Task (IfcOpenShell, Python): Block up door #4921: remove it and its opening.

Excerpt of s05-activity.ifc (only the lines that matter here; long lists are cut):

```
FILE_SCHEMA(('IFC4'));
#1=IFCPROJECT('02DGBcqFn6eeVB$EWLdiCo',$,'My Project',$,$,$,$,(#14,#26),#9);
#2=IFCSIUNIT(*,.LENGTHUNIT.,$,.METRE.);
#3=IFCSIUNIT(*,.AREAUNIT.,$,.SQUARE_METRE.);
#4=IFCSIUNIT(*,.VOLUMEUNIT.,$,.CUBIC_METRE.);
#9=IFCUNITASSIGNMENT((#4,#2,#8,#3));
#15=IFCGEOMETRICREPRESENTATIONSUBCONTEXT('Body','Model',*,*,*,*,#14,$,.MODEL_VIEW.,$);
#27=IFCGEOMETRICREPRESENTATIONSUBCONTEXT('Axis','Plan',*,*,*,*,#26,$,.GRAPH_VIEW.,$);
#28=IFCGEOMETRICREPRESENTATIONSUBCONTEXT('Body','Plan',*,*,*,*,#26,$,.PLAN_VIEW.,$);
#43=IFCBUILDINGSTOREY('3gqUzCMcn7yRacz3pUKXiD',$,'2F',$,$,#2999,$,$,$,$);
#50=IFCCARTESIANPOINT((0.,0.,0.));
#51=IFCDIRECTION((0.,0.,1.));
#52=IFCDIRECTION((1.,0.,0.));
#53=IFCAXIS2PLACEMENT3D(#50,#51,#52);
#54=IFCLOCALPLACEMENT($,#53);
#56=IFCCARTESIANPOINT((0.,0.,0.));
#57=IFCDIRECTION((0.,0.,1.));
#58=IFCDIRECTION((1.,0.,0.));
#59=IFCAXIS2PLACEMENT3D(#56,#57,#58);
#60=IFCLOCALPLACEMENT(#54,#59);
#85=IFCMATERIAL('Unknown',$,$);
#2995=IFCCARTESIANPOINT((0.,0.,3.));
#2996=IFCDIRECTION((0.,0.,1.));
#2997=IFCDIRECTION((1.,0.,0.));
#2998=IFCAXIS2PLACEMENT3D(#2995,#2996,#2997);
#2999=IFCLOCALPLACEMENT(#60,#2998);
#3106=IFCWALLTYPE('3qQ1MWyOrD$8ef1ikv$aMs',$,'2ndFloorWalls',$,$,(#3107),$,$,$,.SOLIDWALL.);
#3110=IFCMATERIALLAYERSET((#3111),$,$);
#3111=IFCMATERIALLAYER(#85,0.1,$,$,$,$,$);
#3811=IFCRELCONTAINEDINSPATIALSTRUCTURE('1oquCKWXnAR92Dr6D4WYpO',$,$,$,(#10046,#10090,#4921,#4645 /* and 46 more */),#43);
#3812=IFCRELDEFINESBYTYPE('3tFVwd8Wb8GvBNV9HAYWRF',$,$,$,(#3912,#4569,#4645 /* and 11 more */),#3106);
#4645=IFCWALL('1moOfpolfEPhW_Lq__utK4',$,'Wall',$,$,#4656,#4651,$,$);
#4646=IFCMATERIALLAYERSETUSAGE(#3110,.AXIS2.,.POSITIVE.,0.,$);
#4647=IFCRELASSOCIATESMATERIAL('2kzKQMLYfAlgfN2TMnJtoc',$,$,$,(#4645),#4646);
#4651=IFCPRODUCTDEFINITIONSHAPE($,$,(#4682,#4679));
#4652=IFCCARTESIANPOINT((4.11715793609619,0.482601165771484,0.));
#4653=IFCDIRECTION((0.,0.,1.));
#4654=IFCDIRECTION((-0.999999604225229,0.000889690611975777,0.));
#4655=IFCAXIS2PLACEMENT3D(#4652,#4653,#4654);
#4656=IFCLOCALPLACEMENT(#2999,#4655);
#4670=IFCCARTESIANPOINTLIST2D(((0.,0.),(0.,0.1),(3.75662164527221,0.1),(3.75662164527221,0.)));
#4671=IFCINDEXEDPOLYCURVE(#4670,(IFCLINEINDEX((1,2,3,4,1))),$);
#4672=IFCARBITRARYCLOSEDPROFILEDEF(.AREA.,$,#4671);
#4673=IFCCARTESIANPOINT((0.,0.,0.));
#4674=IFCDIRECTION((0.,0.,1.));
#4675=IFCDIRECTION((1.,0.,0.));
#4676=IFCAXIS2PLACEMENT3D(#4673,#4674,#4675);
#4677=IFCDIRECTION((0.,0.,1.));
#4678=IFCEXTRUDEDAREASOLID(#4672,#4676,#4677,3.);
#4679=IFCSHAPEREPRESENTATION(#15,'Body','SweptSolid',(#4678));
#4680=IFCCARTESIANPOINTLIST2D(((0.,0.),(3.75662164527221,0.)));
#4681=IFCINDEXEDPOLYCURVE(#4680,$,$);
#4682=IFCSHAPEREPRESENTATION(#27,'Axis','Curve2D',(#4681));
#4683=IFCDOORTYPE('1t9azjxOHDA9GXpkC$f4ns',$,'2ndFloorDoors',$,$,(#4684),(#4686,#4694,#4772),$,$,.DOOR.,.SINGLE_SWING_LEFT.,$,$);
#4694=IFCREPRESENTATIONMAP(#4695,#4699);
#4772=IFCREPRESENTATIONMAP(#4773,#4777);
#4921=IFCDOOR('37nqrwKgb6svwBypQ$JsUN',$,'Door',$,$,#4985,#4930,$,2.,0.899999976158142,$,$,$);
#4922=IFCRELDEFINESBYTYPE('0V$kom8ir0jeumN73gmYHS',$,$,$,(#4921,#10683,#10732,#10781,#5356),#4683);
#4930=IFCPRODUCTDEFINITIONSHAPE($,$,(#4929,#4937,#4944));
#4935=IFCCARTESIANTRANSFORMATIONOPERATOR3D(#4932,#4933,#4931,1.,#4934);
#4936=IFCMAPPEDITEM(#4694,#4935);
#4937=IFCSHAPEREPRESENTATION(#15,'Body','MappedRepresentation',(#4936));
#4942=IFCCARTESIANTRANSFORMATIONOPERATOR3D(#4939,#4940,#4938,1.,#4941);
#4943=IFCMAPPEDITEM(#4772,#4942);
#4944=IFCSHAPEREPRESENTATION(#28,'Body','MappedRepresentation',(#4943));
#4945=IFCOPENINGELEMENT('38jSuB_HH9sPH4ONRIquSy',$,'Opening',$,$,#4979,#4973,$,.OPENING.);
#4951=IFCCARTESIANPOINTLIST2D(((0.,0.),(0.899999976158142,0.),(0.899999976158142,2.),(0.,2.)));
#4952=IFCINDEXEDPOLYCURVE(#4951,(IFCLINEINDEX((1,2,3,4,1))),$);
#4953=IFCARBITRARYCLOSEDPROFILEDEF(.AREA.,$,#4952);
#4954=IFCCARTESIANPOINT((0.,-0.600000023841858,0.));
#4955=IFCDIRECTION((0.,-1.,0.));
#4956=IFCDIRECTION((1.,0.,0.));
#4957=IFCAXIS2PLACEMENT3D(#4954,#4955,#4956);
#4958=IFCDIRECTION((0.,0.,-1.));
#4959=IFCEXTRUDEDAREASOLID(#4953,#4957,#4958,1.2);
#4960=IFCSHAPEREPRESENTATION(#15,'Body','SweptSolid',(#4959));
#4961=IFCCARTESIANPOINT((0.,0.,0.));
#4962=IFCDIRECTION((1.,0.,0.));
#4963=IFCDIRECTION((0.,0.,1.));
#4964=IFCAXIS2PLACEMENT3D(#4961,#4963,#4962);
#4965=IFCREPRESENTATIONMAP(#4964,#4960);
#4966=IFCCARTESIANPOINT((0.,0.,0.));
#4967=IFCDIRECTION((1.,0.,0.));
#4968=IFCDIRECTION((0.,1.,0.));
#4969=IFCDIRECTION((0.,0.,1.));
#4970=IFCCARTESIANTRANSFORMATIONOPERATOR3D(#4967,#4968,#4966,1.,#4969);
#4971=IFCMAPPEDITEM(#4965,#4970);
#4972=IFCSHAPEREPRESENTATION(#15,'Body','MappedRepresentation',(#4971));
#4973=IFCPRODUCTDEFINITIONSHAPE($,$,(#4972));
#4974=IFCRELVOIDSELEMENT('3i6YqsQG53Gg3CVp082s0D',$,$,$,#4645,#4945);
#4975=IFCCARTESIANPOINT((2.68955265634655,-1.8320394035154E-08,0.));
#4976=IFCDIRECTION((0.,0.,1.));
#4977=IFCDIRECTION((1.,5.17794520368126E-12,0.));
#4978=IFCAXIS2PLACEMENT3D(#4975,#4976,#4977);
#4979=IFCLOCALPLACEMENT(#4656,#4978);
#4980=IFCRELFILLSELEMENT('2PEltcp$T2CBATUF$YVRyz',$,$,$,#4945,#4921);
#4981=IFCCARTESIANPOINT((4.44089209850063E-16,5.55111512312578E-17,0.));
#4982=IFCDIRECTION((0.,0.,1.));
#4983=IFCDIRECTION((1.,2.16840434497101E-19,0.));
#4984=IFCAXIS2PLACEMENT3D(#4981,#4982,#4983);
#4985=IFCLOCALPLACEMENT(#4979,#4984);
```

```python
import ifcopenshell
import ifcopenshell.api.feature
import ifcopenshell.api.root
import ifcopenshell.geom
import ifcopenshell.util.shape

model = ifcopenshell.open("s05-activity.ifc")
settings = ifcopenshell.geom.settings()


def volume(element):
    """Net volume in cubic metres, openings subtracted."""
    shape = ifcopenshell.geom.create_shape(settings, element)
    return ifcopenshell.util.shape.get_volume(shape.geometry)


door = model.by_guid("37nqrwKgb6svwBypQ$JsUN")
opening = door.FillsVoids[0].RelatingOpeningElement
wall = opening.VoidsElements[0].RelatingBuildingElement
before = volume(wall)

ifcopenshell.api.root.remove_product(model, product=door)
ifcopenshell.api.feature.remove_feature(model, feature=opening)

after = volume(wall)

print(f"wall volume {before:.3f} -> {after:.3f} m3")

model.write("s05-activity_updated.ifc")
```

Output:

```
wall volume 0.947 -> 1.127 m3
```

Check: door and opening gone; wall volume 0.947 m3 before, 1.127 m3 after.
